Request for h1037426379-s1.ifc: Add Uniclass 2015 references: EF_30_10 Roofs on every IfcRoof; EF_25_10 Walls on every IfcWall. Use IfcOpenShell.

First a look at what the model holds.

```python
import ifcopenshell

model = ifcopenshell.open("h1037426379-s1.ifc")
print(model.schema)
print("classifications:", [c.Name for c in model.by_type("IfcClassification")])
for ifc_class in ("IfcDoor", "IfcRoof", "IfcStair", "IfcWall", "IfcWindow"):
    print(ifc_class, len(model.by_type(ifc_class)))
```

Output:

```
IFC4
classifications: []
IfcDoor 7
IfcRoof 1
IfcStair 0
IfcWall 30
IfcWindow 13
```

```python
import ifcopenshell
import ifcopenshell.api.classification

model = ifcopenshell.open("h1037426379-s1.ifc")

system = ifcopenshell.api.classification.add_classification(model, classification="Uniclass 2015")

codes = {
    "IfcRoof": ("EF_30_10", "Roofs"),
    "IfcWall": ("EF_25_10", "Walls"),
}
for ifc_class, (code, name) in codes.items():
    products = model.by_type(ifc_class)
    ifcopenshell.api.classification.add_reference(
        model, products=products, classification=system, identification=code, name=name
    )
    print(code, len(products))

model.write("h1037426379-s1_edited.ifc")
```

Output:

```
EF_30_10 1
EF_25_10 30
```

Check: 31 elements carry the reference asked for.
